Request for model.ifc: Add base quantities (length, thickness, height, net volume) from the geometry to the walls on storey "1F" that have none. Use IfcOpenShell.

First a look at what the model holds.

```python
import ifcopenshell
import ifcopenshell.util.element
import ifcopenshell.util.unit

model = ifcopenshell.open("model.ifc")
print(model.schema)
for unit_type in ("LENGTHUNIT", "AREAUNIT", "VOLUMEUNIT"):
    print(unit_type, ifcopenshell.util.unit.calculate_unit_scale(model, unit_type))
storey = next(s for s in model.by_type("IfcBuildingStorey") if s.Name == "1F")
walls = [e for e in ifcopenshell.util.element.get_decomposition(storey) if e.is_a("IfcWall")]
for e in sorted(walls, key=lambda e: e.id()):
    print(e.id(), e.is_a(), e.Name, list(ifcopenshell.util.element.get_psets(e, qtos_only=True)), sep=" | ")
```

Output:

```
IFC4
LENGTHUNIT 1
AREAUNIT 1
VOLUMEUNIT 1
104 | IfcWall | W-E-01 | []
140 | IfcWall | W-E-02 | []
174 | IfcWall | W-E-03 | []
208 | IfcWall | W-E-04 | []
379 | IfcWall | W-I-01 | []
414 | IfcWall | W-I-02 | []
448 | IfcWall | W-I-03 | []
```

```python
import ifcopenshell
import ifcopenshell.api.pset
import ifcopenshell.geom
import ifcopenshell.util.element
import ifcopenshell.util.shape
import ifcopenshell.util.unit

model = ifcopenshell.open("model.ifc")
unit_scale = ifcopenshell.util.unit.calculate_unit_scale(model)
volume_scale = ifcopenshell.util.unit.calculate_unit_scale(model, "VOLUMEUNIT")
settings = ifcopenshell.geom.settings()

storey = next(s for s in model.by_type("IfcBuildingStorey") if s.Name == "1F")
walls = [e for e in ifcopenshell.util.element.get_decomposition(storey) if e.is_a("IfcWall")]

for e in sorted(walls, key=lambda e: e.id()):
    if ifcopenshell.util.element.get_psets(e, qtos_only=True, should_inherit=False):
        continue
    # Geometry comes back in metres, in the element's own axes.
    shape = ifcopenshell.geom.create_shape(settings, e)
    values = {
        "Length": ifcopenshell.util.shape.get_x(shape.geometry) / unit_scale,
        "Width": ifcopenshell.util.shape.get_y(shape.geometry) / unit_scale,
        "Height": ifcopenshell.util.shape.get_z(shape.geometry) / unit_scale,
        "NetVolume": ifcopenshell.util.shape.get_volume(shape.geometry) / volume_scale,
    }
    qto = ifcopenshell.api.pset.add_qto(model, product=e, name="Qto_WallBaseQuantities")
    ifcopenshell.api.pset.edit_qto(model, qto=qto, properties=values)
    print(e.id(), {k: round(v, 3) for k, v in values.items()})

model.write("model_edited.ifc")
```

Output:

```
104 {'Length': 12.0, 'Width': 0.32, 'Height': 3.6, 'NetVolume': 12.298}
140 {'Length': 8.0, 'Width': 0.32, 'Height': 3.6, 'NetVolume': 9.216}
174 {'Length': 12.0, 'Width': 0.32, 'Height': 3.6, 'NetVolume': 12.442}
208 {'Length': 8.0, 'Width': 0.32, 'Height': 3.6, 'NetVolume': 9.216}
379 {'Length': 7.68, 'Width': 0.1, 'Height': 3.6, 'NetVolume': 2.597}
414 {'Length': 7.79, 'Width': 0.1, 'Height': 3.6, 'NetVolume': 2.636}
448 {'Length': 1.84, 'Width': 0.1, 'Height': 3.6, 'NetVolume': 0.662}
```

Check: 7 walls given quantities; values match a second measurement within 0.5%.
